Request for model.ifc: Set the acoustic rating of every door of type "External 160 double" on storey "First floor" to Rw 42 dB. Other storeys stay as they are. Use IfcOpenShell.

First a look at what the model holds.

```python
import ifcopenshell
import ifcopenshell.util.element

model = ifcopenshell.open("model.ifc")
print(model.schema)
storey = next(s for s in model.by_type("IfcBuildingStorey") if s.Name == "First floor")
doors = [e for e in ifcopenshell.util.element.get_decomposition(storey) if e.is_a("IfcDoor")]
seen = {}
for e in doors:
    element_type = ifcopenshell.util.element.get_type(e)
    key = (element_type.Name if element_type != e and element_type else None, ifcopenshell.util.element.get_pset(e, "Pset_DoorCommon", "AcousticRating"))
    seen[key] = seen.get(key, 0) + 1
for (name, value), count in sorted(seen.items(), key=str):
    print(count, "x", name, "|", value)
```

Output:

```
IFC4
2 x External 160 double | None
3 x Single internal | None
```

```python
import ifcopenshell
import ifcopenshell.api.pset
import ifcopenshell.util.element

model = ifcopenshell.open("model.ifc")

storey = next(s for s in model.by_type("IfcBuildingStorey") if s.Name == "First floor")
doors = [e for e in ifcopenshell.util.element.get_decomposition(storey) if e.is_a("IfcDoor")]

count = 0
for e in doors:
    element_type = ifcopenshell.util.element.get_type(e)
    if element_type in (None, e) or element_type.Name != "External 160 double":
        continue
    # add_pset returns the element's existing set when there is one.
    pset = ifcopenshell.api.pset.add_pset(model, product=e, name="Pset_DoorCommon")
    ifcopenshell.api.pset.edit_pset(model, pset=pset, properties={"AcousticRating": "Rw 42 dB"})
    count += 1

print(count, "doors updated")

model.write("model_updated.ifc")
```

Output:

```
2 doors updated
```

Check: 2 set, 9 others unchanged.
